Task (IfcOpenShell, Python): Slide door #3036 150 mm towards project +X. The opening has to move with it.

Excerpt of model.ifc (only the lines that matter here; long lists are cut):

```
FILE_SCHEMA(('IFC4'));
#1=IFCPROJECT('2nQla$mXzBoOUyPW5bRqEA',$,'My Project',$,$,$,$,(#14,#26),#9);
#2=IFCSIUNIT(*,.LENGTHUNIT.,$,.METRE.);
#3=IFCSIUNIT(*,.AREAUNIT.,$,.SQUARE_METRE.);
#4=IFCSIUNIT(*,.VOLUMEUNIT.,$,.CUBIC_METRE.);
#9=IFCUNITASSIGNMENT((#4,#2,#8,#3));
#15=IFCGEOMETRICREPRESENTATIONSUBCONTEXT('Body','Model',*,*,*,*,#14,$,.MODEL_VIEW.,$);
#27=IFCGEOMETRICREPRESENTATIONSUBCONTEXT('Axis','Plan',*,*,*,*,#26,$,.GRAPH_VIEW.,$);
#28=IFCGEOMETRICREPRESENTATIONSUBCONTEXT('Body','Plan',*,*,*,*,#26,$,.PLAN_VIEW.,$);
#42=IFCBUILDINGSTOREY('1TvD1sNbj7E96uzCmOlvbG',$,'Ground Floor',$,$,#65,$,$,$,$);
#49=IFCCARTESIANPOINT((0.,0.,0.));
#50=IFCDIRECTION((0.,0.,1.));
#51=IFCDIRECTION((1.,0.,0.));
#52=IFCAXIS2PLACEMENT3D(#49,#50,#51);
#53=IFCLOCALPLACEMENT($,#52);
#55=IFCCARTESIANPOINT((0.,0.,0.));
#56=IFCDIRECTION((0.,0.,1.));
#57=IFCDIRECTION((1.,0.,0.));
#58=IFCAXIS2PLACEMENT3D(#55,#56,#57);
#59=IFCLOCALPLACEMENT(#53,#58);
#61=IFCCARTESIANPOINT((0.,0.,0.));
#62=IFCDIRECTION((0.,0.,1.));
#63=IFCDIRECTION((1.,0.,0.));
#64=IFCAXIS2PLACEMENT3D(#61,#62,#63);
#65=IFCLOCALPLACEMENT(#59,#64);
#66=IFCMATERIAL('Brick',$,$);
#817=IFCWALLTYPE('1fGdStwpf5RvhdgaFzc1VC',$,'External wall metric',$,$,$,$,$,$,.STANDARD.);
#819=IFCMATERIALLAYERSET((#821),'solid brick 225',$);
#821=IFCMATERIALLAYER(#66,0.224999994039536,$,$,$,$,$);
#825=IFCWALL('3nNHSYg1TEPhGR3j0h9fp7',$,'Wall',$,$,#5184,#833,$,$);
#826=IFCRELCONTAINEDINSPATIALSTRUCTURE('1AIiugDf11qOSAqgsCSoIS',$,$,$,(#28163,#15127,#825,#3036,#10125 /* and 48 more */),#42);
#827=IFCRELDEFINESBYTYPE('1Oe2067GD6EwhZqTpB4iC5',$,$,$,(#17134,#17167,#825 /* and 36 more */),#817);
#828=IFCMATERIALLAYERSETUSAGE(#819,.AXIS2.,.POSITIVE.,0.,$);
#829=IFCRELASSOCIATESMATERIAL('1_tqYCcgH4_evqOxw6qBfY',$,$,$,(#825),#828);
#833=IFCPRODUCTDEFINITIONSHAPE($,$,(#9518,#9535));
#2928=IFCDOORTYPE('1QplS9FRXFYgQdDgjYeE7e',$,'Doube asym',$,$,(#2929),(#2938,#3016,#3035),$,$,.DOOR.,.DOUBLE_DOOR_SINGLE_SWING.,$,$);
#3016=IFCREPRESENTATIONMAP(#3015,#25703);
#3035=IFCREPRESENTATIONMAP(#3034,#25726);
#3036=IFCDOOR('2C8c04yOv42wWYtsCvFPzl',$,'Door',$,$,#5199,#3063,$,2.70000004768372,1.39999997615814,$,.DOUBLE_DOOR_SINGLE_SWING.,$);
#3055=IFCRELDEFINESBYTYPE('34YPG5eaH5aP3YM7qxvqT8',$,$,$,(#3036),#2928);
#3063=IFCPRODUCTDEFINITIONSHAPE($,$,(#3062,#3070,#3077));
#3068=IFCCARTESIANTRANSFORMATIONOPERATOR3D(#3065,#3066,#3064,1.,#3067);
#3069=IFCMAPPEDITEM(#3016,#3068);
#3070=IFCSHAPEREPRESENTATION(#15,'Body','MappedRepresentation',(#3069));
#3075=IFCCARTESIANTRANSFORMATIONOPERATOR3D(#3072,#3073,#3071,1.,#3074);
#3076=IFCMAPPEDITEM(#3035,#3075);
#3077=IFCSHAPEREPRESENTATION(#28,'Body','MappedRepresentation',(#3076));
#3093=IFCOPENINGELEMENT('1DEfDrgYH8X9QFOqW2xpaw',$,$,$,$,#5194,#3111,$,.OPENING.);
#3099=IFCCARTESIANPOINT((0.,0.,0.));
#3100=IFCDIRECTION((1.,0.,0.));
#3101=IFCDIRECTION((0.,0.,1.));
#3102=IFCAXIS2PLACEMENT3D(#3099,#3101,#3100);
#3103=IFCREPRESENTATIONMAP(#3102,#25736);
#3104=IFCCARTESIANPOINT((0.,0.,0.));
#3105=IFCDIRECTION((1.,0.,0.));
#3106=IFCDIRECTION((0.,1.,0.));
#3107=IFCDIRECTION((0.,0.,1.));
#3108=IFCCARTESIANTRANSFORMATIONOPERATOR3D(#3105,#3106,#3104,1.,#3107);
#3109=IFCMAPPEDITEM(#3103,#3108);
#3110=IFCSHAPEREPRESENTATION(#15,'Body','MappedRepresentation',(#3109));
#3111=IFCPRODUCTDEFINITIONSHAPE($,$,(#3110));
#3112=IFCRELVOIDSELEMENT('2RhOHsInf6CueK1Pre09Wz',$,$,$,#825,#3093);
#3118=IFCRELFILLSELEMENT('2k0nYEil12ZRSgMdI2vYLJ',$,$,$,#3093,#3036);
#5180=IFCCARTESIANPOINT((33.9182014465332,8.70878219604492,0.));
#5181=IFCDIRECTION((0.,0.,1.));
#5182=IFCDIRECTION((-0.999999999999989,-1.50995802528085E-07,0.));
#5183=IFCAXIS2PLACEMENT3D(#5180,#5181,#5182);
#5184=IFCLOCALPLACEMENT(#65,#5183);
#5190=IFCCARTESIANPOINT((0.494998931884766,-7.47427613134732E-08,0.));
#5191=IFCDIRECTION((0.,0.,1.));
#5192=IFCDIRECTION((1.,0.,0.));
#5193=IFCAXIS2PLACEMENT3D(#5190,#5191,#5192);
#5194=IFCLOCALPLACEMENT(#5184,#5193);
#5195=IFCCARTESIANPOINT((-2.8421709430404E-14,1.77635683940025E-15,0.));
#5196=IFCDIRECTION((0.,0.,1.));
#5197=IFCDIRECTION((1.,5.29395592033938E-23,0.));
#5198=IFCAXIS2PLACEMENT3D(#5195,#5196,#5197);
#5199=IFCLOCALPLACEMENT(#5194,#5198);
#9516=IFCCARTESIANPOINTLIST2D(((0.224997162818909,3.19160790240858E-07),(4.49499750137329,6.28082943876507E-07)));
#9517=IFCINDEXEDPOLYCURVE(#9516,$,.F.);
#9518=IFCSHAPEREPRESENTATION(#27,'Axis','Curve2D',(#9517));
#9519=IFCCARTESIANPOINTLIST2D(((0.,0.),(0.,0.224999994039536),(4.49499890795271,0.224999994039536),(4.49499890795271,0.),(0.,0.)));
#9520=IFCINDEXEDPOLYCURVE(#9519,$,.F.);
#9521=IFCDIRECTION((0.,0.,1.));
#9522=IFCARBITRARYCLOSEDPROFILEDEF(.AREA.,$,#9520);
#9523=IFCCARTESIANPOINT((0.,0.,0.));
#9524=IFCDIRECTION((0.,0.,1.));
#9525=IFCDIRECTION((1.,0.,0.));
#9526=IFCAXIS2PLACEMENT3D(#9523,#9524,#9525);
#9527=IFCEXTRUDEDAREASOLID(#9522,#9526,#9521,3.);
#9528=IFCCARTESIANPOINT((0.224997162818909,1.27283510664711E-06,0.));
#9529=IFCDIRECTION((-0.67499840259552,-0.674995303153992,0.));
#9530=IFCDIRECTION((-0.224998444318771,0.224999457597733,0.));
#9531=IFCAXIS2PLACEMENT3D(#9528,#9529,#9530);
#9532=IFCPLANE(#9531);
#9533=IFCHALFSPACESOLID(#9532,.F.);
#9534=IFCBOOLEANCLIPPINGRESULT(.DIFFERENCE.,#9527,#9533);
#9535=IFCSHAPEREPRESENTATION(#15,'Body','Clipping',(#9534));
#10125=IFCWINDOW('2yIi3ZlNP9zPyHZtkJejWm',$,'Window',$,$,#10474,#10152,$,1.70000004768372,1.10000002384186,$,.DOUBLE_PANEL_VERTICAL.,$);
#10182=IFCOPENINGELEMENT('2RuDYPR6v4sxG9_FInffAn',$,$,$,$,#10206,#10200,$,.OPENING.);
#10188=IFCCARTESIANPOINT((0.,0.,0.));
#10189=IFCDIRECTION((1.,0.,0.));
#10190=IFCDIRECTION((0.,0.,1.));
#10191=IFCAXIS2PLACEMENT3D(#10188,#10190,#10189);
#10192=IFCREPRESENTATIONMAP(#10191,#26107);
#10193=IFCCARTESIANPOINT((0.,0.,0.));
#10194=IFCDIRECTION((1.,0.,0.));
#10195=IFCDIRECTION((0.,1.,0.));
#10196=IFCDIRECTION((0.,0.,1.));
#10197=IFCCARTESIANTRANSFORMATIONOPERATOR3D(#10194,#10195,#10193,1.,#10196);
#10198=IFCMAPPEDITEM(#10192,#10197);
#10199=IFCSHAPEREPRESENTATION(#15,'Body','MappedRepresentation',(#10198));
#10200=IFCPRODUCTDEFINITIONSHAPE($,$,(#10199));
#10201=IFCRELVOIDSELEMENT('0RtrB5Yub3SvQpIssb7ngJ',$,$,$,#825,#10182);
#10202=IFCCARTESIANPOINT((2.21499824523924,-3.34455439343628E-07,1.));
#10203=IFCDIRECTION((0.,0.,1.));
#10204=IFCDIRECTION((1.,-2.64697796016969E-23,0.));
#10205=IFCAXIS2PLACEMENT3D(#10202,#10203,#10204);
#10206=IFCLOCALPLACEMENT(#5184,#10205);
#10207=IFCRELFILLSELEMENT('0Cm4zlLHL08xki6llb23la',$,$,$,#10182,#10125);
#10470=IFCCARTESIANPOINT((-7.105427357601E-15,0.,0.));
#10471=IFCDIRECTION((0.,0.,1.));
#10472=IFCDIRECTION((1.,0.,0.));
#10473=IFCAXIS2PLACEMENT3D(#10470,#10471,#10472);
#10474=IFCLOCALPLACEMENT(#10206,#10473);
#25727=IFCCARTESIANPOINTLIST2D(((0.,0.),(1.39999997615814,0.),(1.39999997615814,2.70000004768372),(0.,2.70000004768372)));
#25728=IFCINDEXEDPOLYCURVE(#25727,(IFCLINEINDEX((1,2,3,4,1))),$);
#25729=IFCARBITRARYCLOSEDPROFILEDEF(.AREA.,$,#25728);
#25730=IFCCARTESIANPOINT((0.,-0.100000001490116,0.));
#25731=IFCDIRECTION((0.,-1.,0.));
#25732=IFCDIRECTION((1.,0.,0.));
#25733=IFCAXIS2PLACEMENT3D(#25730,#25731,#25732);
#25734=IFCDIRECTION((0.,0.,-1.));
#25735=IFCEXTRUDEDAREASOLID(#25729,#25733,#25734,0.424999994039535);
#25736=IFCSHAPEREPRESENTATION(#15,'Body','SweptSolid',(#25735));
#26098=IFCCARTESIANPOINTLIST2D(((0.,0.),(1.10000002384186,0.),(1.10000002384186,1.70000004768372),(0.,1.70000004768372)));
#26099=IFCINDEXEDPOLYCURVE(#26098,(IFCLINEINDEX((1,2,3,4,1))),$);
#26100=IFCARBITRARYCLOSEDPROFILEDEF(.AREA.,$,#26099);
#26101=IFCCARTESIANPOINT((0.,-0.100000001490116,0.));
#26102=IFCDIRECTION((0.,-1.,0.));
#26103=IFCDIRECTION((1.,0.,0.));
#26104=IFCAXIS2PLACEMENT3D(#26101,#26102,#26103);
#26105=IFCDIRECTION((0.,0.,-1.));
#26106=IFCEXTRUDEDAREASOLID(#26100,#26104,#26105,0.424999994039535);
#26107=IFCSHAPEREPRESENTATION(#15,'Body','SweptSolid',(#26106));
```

```python
import ifcopenshell
import ifcopenshell.api.geometry
import ifcopenshell.util.placement

model = ifcopenshell.open("model.ifc")

door = model.by_guid("2C8c04yOv42wWYtsCvFPzl")
opening = door.FillsVoids[0].RelatingOpeningElement
wall = opening.VoidsElements[0].RelatingBuildingElement

wall_matrix = ifcopenshell.util.placement.get_local_placement(wall.ObjectPlacement)
shift = wall_matrix[:3, 0] * -0.15
before = ifcopenshell.util.placement.get_local_placement(door.ObjectPlacement)[:3, 3].copy()

# The door is placed relative to its opening, so it follows when the opening moves.
matrix = ifcopenshell.util.placement.get_local_placement(opening.ObjectPlacement)
matrix[:3, 3] += shift
ifcopenshell.api.geometry.edit_object_placement(
    model, product=opening, matrix=matrix, is_si=False, should_transform_children=True
)

after = ifcopenshell.util.placement.get_local_placement(door.ObjectPlacement)[:3, 3]
print("door moved by", (after - before).round(3) + 0.0)

model.write("model_updated.ifc")
```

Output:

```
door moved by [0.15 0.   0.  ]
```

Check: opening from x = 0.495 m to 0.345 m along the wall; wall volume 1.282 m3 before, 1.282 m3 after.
